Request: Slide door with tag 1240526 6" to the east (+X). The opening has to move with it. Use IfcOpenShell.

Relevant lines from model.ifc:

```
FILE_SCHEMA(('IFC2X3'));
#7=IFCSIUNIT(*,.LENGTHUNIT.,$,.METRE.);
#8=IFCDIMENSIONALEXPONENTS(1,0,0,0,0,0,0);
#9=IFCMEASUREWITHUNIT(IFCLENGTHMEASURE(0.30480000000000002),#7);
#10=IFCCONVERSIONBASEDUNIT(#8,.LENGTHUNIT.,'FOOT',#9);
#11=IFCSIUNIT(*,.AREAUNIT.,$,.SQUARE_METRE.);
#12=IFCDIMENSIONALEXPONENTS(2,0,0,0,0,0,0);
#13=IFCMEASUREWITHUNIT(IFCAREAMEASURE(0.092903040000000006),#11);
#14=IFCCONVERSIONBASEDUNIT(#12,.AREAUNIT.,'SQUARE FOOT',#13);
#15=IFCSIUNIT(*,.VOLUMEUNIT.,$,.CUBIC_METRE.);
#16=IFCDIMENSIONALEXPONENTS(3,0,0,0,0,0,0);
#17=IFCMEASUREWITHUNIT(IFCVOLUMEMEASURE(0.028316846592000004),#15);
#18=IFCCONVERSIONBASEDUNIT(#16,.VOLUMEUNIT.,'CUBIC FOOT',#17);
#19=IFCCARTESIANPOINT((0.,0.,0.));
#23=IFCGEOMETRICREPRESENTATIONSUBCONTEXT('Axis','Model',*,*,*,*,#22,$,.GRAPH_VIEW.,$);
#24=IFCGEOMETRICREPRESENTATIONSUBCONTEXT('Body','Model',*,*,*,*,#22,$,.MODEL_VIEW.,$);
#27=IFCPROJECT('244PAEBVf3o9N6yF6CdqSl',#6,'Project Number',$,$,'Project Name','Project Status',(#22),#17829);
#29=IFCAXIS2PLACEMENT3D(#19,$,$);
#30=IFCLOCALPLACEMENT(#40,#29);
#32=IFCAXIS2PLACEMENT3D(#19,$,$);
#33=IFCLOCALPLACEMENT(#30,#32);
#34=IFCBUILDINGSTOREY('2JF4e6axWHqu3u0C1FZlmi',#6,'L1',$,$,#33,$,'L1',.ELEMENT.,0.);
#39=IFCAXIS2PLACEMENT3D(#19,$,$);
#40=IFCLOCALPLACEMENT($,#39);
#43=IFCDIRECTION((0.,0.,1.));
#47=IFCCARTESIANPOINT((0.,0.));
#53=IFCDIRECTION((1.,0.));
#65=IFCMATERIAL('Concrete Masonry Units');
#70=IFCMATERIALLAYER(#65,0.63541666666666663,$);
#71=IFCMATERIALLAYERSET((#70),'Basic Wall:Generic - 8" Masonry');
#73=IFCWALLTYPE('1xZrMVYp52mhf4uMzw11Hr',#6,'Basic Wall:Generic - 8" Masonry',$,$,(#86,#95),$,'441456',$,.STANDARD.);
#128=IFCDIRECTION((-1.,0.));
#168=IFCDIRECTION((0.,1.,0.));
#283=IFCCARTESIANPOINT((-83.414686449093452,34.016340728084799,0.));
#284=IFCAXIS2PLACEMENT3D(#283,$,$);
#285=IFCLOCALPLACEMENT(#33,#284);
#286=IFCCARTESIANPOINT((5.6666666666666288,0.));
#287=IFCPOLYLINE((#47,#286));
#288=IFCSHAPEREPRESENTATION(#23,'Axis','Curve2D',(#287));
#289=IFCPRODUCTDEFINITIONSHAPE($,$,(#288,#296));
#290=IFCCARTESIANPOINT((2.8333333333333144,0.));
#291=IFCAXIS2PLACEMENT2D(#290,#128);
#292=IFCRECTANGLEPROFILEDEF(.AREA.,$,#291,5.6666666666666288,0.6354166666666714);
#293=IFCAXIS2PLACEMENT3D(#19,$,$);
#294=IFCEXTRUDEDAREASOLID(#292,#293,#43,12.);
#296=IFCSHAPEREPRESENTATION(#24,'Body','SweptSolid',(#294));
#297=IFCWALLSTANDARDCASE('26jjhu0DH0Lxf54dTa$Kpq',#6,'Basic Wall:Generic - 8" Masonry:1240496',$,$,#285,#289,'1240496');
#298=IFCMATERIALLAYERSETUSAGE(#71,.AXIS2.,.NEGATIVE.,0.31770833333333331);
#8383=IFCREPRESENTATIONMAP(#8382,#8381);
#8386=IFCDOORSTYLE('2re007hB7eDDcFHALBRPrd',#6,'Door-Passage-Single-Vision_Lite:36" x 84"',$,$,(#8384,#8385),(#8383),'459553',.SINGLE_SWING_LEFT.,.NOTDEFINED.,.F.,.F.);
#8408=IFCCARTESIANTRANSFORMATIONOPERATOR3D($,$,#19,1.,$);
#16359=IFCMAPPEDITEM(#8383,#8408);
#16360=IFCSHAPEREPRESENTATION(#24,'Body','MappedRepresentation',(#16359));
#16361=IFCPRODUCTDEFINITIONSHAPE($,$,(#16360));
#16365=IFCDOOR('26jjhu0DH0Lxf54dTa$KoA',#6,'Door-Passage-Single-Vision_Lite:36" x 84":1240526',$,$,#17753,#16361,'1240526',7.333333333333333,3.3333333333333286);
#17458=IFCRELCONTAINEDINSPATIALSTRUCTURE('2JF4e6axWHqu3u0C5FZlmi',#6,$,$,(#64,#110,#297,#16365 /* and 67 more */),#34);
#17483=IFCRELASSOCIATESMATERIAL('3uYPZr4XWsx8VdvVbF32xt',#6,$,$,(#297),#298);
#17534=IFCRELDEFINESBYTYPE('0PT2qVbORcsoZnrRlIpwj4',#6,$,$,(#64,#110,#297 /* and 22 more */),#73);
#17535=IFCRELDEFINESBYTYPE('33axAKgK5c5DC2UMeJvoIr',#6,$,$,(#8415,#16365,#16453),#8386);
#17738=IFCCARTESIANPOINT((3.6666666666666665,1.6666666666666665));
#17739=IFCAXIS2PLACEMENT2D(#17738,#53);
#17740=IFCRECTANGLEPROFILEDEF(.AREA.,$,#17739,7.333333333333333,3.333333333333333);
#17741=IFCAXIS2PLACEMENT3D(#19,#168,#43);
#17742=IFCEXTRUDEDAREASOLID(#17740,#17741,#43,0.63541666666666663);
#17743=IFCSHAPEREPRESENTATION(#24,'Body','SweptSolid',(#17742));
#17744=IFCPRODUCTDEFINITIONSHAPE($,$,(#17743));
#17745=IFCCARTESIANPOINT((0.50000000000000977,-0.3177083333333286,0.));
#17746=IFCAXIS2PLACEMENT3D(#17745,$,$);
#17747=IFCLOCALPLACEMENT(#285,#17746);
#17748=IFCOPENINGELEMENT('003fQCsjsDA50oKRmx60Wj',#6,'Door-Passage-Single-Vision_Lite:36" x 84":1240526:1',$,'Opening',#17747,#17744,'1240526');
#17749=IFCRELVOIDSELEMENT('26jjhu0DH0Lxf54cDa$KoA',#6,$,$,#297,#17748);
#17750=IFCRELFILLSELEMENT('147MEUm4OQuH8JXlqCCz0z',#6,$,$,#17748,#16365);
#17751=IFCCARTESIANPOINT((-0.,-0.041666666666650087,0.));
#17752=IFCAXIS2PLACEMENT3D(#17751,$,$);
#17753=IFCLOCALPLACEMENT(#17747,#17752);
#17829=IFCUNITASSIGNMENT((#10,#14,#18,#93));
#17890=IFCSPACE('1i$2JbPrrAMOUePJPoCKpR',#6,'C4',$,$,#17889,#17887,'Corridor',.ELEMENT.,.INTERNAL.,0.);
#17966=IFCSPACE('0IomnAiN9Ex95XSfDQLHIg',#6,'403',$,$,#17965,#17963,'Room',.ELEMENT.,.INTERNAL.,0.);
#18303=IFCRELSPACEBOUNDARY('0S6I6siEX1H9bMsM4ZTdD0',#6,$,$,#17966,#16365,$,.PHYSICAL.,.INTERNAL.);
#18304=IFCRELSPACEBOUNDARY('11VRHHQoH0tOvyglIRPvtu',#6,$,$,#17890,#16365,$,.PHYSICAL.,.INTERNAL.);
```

```python
import ifcopenshell
import ifcopenshell.api.geometry
import ifcopenshell.util.placement
import ifcopenshell.util.unit

model = ifcopenshell.open("model.ifc")
unit_scale = ifcopenshell.util.unit.calculate_unit_scale(model)

door = model.by_guid("26jjhu0DH0Lxf54dTa$KoA")
opening = door.FillsVoids[0].RelatingOpeningElement
wall = opening.VoidsElements[0].RelatingBuildingElement

wall_matrix = ifcopenshell.util.placement.get_local_placement(wall.ObjectPlacement)
shift = wall_matrix[:3, 0] * 6 * 0.0254 / unit_scale
before = ifcopenshell.util.placement.get_local_placement(door.ObjectPlacement)[:3, 3].copy()

# The door is placed relative to its opening, so it follows when the opening moves.
matrix = ifcopenshell.util.placement.get_local_placement(opening.ObjectPlacement)
matrix[:3, 3] += shift
ifcopenshell.api.geometry.edit_object_placement(
    model, product=opening, matrix=matrix, is_si=False, should_transform_children=True
)

after = ifcopenshell.util.placement.get_local_placement(door.ObjectPlacement)[:3, 3]
print("door moved by", (after - before).round(3) + 0.0)

model.write("model-out.ifc")
```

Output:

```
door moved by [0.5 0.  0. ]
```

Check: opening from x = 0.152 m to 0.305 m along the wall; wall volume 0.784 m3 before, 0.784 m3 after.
